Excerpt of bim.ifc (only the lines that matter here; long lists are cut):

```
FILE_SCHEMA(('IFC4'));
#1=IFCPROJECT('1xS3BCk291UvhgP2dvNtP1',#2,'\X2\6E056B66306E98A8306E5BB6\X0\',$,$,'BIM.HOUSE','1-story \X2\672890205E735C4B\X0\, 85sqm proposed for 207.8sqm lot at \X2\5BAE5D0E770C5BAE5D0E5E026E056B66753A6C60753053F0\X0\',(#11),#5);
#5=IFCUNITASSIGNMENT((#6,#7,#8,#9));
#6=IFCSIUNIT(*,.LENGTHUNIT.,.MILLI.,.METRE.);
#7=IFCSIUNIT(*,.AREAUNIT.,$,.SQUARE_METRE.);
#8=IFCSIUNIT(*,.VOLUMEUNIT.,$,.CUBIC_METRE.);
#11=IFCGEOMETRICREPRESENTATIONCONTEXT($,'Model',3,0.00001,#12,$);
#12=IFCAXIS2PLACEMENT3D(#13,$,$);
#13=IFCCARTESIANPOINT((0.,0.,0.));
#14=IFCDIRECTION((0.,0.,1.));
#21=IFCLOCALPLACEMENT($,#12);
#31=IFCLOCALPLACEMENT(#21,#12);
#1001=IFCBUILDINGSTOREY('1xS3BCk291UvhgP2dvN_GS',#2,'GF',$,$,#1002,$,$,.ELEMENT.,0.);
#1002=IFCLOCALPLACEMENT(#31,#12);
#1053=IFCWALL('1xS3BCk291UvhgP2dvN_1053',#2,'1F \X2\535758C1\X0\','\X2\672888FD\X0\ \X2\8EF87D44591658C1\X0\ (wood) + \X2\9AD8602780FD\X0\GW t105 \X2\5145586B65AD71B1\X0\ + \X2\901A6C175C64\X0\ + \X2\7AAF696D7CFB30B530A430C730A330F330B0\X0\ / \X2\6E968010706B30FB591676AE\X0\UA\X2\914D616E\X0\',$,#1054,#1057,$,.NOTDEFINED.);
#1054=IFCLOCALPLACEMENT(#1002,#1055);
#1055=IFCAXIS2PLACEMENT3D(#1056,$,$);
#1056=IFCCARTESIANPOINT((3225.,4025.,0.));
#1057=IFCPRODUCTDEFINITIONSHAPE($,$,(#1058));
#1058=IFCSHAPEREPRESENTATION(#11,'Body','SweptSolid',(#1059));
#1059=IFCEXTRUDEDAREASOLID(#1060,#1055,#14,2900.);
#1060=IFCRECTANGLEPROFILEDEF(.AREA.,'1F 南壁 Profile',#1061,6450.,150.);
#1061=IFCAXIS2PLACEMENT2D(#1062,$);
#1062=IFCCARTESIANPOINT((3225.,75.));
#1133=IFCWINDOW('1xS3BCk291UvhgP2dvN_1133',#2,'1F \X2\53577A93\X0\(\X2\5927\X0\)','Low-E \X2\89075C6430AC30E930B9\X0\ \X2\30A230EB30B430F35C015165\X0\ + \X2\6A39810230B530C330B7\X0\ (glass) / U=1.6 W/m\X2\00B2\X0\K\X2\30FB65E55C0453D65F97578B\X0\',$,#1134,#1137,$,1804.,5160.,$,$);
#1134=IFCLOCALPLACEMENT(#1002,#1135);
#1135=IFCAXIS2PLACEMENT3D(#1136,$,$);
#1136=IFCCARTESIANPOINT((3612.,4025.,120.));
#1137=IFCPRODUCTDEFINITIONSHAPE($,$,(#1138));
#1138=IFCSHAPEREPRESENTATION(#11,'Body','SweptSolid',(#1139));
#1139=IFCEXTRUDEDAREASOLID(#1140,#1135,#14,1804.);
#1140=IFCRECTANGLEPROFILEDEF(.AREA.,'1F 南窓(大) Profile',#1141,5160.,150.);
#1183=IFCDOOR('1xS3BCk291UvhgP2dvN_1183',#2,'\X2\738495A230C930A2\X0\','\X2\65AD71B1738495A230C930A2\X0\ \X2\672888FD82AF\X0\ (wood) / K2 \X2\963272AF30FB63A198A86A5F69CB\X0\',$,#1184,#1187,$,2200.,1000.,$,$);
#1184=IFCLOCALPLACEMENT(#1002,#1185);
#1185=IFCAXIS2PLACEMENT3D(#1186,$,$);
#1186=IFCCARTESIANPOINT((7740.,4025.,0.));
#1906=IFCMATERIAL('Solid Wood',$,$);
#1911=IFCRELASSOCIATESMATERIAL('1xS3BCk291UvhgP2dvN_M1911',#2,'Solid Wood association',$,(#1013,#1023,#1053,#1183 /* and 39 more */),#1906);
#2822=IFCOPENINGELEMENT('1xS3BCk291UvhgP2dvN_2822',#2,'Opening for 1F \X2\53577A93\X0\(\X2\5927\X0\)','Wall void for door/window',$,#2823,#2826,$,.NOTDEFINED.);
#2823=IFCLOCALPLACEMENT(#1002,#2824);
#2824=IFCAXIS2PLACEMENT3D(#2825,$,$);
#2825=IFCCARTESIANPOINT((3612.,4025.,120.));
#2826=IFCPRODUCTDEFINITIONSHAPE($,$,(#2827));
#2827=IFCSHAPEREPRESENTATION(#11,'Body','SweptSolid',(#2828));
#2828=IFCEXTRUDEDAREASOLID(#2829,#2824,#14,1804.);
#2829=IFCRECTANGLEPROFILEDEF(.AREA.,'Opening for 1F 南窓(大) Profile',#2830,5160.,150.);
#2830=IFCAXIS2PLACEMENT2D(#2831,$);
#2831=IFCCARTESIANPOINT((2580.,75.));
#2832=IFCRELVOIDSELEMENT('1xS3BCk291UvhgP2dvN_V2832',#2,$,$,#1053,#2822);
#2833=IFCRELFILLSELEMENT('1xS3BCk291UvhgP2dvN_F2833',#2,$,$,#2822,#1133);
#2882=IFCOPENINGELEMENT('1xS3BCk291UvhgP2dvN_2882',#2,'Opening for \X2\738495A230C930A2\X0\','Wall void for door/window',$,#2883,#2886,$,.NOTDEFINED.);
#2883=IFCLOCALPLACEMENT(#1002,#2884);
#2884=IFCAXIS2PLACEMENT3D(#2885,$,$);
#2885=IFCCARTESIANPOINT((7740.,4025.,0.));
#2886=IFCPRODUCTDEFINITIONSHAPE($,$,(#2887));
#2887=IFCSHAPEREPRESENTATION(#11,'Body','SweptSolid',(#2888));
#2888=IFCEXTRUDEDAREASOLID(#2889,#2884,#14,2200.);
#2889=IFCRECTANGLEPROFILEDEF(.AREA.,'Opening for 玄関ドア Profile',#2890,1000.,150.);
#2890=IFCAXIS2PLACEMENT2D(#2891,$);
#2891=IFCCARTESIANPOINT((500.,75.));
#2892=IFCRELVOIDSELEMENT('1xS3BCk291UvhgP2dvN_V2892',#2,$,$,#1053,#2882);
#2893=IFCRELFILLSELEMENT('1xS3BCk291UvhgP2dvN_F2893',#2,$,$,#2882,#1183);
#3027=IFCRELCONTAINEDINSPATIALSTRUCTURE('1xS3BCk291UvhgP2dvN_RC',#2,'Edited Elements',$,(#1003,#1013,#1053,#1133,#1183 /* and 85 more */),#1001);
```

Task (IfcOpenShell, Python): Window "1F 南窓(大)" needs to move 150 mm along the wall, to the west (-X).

```python
import ifcopenshell
import ifcopenshell.api.geometry
import ifcopenshell.util.placement

model = ifcopenshell.open("bim.ifc")

window = model.by_guid("1xS3BCk291UvhgP2dvN_1133")
opening = window.FillsVoids[0].RelatingOpeningElement
wall = opening.VoidsElements[0].RelatingBuildingElement

wall_matrix = ifcopenshell.util.placement.get_local_placement(wall.ObjectPlacement)
shift = wall_matrix[:3, 0] * -150.0
before = ifcopenshell.util.placement.get_local_placement(window.ObjectPlacement)[:3, 3].copy()

# The window is not placed relative to its opening, so move both.
for product in (opening, window):
    matrix = ifcopenshell.util.placement.get_local_placement(product.ObjectPlacement)
    matrix[:3, 3] += shift
    ifcopenshell.api.geometry.edit_object_placement(model, product=product, matrix=matrix, is_si=False)

after = ifcopenshell.util.placement.get_local_placement(window.ObjectPlacement)[:3, 3]
print("window moved by", (after - before).round(3) + 0.0)

model.write("bim-out.ifc")
```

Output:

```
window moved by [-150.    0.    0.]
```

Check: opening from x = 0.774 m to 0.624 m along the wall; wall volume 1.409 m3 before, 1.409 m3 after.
